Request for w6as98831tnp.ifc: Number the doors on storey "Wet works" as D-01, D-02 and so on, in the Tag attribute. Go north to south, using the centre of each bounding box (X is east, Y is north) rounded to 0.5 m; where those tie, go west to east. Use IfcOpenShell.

First a look at what the model holds.

```python
import ifcopenshell
import ifcopenshell.util.element
import ifcopenshell.util.placement

model = ifcopenshell.open("w6as98831tnp.ifc")
print(model.schema)
storey = next(s for s in model.by_type("IfcBuildingStorey") if s.Name == "Wet works")
doors = [e for e in ifcopenshell.util.element.get_decomposition(storey) if e.is_a("IfcDoor")]
for e in sorted(doors, key=lambda e: e.id()):
    origin = ifcopenshell.util.placement.get_local_placement(e.ObjectPlacement)[:3, 3]
    print(e.id(), e.Tag, e.Name, origin.round(2) + 0.0, sep=" | ")
```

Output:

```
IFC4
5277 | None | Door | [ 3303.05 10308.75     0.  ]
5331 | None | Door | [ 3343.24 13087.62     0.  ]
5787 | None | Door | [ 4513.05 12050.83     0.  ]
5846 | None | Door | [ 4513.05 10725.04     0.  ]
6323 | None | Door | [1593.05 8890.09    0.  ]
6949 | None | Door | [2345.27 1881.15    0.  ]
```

```python
import ifcopenshell
import ifcopenshell.geom
import ifcopenshell.util.element
import ifcopenshell.util.shape

model = ifcopenshell.open("w6as98831tnp.ifc")
settings = ifcopenshell.geom.settings()
settings.set("use-world-coords", True)


def centre(element):
    shape = ifcopenshell.geom.create_shape(settings, element)
    return ifcopenshell.util.shape.get_bbox_centroid(shape.geometry)


storey = next(s for s in model.by_type("IfcBuildingStorey") if s.Name == "Wet works")
doors = [e for e in ifcopenshell.util.element.get_decomposition(storey) if e.is_a("IfcDoor")]

# Insertion points can sit at a corner or the storey origin, so sort by the geometry (in metres).
centres = {e: centre(e) for e in doors}
doors.sort(key=lambda e: (-round(centres[e][1] / 0.5), centres[e][0]))

for i, e in enumerate(doors, start=1):
    number = f"D-{i:02d}"
    e.Tag = number
    print(e.id(), number)

model.write("w6as98831tnp_v2.ifc")
```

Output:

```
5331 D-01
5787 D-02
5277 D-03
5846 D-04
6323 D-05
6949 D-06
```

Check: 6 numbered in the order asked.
